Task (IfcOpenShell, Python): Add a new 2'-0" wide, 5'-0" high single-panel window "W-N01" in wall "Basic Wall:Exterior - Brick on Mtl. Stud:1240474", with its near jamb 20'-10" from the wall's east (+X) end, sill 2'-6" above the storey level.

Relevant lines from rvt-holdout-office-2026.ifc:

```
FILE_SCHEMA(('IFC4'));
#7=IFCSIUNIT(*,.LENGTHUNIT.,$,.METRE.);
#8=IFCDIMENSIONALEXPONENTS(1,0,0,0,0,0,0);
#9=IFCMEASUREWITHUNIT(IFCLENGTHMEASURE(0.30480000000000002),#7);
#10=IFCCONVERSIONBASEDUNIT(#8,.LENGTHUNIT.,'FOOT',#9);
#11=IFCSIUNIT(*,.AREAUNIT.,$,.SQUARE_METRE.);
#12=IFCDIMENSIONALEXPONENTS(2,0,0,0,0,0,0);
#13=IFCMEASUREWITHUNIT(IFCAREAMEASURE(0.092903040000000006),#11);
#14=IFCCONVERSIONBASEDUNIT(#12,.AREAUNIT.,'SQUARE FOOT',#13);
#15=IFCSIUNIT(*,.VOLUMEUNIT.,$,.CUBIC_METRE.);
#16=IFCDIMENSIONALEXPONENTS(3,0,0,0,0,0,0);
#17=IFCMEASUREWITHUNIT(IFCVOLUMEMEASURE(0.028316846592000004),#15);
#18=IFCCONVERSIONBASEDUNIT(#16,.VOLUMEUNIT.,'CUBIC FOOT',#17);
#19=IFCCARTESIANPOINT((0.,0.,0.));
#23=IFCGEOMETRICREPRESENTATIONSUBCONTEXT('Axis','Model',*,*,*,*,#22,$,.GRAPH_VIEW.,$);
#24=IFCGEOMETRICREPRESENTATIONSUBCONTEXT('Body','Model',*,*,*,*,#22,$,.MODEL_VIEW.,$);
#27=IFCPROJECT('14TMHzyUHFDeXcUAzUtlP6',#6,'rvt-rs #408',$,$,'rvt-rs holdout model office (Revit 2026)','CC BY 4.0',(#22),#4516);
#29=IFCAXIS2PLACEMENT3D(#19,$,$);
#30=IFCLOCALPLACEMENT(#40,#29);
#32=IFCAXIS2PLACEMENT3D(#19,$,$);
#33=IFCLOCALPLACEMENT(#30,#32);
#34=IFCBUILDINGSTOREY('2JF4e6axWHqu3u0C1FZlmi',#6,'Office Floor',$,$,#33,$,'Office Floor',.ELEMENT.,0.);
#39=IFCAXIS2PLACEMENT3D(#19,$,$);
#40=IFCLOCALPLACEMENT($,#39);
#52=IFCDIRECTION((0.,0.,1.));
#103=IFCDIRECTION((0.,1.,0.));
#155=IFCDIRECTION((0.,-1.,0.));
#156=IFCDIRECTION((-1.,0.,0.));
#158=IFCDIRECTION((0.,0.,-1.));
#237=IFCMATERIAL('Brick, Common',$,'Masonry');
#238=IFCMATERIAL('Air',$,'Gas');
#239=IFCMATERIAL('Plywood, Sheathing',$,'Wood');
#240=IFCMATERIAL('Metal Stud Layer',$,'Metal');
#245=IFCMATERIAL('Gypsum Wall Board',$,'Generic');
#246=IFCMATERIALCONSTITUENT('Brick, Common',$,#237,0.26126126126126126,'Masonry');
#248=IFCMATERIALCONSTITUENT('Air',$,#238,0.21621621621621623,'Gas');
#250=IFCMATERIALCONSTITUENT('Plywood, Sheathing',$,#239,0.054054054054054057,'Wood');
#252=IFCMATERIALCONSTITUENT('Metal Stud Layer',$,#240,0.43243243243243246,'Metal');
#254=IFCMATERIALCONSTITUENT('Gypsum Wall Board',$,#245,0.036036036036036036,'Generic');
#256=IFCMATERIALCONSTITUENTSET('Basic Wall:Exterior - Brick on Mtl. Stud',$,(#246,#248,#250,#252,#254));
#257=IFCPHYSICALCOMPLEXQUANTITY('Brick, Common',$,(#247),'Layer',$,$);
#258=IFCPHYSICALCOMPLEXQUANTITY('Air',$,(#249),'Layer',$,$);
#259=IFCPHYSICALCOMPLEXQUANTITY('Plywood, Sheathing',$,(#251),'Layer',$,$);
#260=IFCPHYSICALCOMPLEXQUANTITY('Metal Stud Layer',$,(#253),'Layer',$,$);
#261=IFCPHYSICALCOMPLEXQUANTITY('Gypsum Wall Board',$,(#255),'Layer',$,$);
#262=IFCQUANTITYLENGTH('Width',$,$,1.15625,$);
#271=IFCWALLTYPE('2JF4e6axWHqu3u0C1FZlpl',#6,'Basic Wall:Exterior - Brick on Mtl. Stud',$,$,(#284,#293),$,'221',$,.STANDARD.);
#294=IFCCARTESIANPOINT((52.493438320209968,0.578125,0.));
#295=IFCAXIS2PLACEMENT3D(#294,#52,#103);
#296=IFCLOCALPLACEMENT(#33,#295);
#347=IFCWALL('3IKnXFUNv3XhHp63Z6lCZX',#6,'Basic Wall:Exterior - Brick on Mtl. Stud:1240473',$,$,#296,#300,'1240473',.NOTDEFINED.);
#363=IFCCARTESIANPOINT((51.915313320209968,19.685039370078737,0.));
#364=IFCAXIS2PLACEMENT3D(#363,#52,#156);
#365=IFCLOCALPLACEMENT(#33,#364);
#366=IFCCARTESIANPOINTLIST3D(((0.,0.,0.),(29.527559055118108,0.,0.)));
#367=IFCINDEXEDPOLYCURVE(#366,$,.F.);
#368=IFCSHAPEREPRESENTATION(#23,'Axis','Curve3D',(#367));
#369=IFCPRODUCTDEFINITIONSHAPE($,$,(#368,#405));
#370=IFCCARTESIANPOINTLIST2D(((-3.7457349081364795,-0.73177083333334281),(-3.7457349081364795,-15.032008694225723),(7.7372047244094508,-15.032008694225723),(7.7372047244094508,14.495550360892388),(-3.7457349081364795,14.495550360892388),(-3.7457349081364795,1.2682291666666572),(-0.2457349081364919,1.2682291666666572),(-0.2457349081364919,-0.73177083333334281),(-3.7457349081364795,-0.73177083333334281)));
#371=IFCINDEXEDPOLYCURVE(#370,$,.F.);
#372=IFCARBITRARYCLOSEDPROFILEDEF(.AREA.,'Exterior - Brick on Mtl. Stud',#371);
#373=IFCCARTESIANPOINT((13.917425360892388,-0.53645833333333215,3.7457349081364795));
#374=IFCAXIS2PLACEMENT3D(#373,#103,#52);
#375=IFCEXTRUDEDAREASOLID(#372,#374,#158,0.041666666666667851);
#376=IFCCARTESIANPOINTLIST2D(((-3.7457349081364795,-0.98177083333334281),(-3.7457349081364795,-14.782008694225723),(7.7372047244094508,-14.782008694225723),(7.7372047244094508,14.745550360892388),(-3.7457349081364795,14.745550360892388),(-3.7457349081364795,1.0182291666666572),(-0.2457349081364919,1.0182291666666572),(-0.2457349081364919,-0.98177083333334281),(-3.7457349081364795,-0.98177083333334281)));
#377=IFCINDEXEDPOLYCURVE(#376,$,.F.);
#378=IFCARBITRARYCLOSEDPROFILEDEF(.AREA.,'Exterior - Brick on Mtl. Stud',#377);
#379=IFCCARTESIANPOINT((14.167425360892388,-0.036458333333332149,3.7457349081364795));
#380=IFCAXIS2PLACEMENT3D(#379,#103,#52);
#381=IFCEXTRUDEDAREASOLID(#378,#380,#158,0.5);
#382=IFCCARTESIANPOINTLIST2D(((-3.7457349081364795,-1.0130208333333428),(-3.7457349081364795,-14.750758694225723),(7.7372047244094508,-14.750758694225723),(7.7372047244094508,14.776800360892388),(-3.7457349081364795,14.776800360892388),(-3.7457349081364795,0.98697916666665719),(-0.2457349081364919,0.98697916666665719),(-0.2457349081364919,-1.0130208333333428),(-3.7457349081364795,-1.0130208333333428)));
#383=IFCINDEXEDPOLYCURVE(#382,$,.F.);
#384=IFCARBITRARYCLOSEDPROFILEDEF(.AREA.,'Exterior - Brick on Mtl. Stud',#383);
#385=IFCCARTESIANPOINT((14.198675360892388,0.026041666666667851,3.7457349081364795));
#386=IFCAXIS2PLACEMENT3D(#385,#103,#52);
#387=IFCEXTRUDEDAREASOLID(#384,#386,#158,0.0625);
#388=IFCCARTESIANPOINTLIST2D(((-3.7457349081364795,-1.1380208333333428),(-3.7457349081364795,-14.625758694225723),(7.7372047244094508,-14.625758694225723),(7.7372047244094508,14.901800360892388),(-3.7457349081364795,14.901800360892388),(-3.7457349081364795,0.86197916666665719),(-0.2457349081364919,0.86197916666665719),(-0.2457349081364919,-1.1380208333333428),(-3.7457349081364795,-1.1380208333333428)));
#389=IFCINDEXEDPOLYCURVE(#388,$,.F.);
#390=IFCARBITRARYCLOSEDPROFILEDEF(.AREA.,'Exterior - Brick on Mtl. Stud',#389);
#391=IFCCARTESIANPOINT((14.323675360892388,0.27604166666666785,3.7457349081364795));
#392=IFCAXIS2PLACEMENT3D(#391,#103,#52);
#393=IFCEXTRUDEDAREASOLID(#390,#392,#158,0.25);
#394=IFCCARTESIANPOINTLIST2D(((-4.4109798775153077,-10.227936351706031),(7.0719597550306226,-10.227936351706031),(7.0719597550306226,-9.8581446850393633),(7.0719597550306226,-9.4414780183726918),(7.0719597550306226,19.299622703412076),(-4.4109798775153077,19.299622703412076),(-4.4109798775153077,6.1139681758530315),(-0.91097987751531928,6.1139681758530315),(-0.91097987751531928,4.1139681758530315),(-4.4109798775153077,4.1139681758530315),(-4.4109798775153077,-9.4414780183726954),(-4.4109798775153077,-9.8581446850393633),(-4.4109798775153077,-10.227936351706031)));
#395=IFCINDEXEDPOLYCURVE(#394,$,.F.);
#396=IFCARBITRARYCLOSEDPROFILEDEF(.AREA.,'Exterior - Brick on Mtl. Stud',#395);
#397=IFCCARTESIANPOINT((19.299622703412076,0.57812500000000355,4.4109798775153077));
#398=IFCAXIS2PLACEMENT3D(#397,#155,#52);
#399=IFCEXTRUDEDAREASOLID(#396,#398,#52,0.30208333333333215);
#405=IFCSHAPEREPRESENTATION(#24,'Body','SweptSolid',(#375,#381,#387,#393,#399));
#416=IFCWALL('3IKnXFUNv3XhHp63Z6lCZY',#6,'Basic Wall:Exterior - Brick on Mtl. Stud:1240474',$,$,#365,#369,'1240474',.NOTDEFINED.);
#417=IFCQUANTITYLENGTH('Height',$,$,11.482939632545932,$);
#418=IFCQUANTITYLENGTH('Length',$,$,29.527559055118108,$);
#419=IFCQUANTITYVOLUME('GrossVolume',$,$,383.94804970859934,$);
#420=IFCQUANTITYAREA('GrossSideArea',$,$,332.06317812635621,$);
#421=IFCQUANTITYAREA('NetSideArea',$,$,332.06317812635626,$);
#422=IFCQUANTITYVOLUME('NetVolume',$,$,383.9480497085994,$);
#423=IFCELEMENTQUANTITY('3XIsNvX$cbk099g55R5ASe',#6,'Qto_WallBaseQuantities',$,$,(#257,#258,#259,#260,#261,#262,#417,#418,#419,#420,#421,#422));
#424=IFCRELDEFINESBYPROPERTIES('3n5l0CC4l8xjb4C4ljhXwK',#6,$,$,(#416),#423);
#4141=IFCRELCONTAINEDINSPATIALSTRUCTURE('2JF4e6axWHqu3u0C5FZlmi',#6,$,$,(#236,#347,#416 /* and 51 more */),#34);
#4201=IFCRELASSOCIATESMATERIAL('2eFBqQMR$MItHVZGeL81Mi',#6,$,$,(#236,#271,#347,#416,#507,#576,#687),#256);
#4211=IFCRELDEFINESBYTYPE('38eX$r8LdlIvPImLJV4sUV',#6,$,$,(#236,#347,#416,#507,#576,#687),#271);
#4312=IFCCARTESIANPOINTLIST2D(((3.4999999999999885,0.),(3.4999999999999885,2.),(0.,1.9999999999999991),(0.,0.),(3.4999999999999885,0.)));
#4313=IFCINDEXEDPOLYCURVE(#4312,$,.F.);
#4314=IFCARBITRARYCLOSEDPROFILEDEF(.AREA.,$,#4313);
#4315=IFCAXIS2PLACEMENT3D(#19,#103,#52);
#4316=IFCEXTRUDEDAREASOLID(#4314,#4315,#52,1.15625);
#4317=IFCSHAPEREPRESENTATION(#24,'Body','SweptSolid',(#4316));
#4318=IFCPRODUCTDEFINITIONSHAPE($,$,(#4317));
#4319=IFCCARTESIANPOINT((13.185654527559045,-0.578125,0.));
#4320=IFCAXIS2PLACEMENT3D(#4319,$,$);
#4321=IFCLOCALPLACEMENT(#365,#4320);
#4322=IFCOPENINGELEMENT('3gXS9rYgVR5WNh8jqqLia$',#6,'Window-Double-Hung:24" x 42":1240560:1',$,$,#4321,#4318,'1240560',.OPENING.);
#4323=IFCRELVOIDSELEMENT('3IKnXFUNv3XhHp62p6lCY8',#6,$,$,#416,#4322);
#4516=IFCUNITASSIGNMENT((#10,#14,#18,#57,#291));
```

```python
import numpy as np
import ifcopenshell
import ifcopenshell.api.feature
import ifcopenshell.api.geometry
import ifcopenshell.api.pset
import ifcopenshell.api.root
import ifcopenshell.api.spatial
import ifcopenshell.geom
import ifcopenshell.util.element
import ifcopenshell.util.placement
import ifcopenshell.util.representation
import ifcopenshell.util.shape
import ifcopenshell.util.unit

model = ifcopenshell.open("rvt-holdout-office-2026.ifc")
unit_scale = ifcopenshell.util.unit.calculate_unit_scale(model)
area_scale = ifcopenshell.util.unit.calculate_unit_scale(model, "AREAUNIT")
volume_scale = ifcopenshell.util.unit.calculate_unit_scale(model, "VOLUMEUNIT")
settings = ifcopenshell.geom.settings()


def volume(element):
    """Net volume in cubic metres, openings subtracted."""
    shape = ifcopenshell.geom.create_shape(settings, element)
    return ifcopenshell.util.shape.get_volume(shape.geometry)


wall = model.by_id(416)
storey = ifcopenshell.util.element.get_container(wall, ifc_class="IfcBuildingStorey")
context = ifcopenshell.util.representation.get_context(model, "Model", "Body", "MODEL_VIEW")
before = volume(wall)

width, height, from_end, sill = 0.6096, 1.524, 6.35, 0.762  # metres

# The wall runs along its own X axis, and the end named is its -X end.
wall_shape = ifcopenshell.geom.create_shape(settings, wall)
x, y, z = ifcopenshell.util.shape.get_vertices(wall_shape.geometry).T
start = x.min() + from_end
face, thickness = float(y.min()), float(y.max() - y.min())
wall_matrix = ifcopenshell.util.placement.get_local_placement(wall.ObjectPlacement)
level = ifcopenshell.util.placement.get_local_placement(storey.ObjectPlacement)[2, 3]


def in_wall(x, y):
    """Placement at x, y metres in the wall's axes, at sill height."""
    matrix = wall_matrix.copy()
    matrix[:, 3] = wall_matrix @ np.array([x / unit_scale, y / unit_scale, 0.0, 1.0])
    matrix[2, 3] = level + sill / unit_scale
    return matrix


# Opening: a box that overshoots both wall faces by 50 mm.
opening = ifcopenshell.api.root.create_entity(model, ifc_class="IfcOpeningElement", predefined_type="OPENING")
box = ifcopenshell.api.geometry.add_wall_representation(
    model, context=context, length=width, height=height, thickness=thickness + 0.1
)
ifcopenshell.api.geometry.assign_representation(model, product=opening, representation=box)
ifcopenshell.api.geometry.edit_object_placement(model, product=opening, matrix=in_wall(start, face - 0.05), is_si=False)
ifcopenshell.api.feature.add_feature(model, feature=opening, element=wall)

window = ifcopenshell.api.root.create_entity(model, ifc_class="IfcWindow", name="W-N01", predefined_type="WINDOW")
window.OverallWidth, window.OverallHeight = width / unit_scale, height / unit_scale
window.PartitioningType = "SINGLE_PANEL"
body = ifcopenshell.api.geometry.add_window_representation(
    model,
    context=context,
    overall_width=window.OverallWidth,
    overall_height=window.OverallHeight,
    partition_type="SINGLE_PANEL",
)
ifcopenshell.api.geometry.assign_representation(model, product=window, representation=body)
ifcopenshell.api.spatial.assign_container(model, products=[window], relating_structure=storey)
ifcopenshell.api.feature.add_filling(model, opening=opening, element=window)

# Centre the window in the wall's thickness.
ifcopenshell.api.geometry.edit_object_placement(model, product=window, matrix=in_wall(start, face), is_si=False)
window_shape = ifcopenshell.geom.create_shape(settings, window)
depth = ifcopenshell.util.shape.get_vertices(window_shape.geometry)[:, 1]
offset = face + thickness / 2 - (depth.min() + depth.max()) / 2
ifcopenshell.api.geometry.edit_object_placement(model, product=window, matrix=in_wall(start, offset), is_si=False)

after = volume(wall)

# Update the wall's stored quantities.
qto = model.by_id(ifcopenshell.util.element.get_pset(wall, "Qto_WallBaseQuantities", should_inherit=False)["id"])
ifcopenshell.api.pset.edit_qto(model, qto=qto, properties={
    "NetSideArea": after / thickness / area_scale,
    "NetVolume": after / volume_scale,
})

print(f"wall volume {before:.3f} -> {after:.3f} m3")

model.write("rvt-holdout-office-2026-out.ifc")
```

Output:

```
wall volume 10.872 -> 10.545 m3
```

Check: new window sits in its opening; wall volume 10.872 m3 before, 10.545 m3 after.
